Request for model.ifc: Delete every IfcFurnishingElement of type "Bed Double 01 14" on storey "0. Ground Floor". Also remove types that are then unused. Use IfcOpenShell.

First a look at what the model holds.

```python
import ifcopenshell
import ifcopenshell.util.element

model = ifcopenshell.open("model.ifc")
print(model.schema)
storey = next(s for s in model.by_type("IfcBuildingStorey") if s.Name == "0. Ground Floor")
furniture = [e for e in ifcopenshell.util.element.get_decomposition(storey) if e.is_a("IfcFurnishingElement")]
seen = {}
for e in furniture:
    element_type = ifcopenshell.util.element.get_type(e)
    name = element_type.Name if element_type not in (None, e) else None
    seen[name] = seen.get(name, 0) + 1
for name, count in sorted(seen.items(), key=str):
    print(count, "x", name)
```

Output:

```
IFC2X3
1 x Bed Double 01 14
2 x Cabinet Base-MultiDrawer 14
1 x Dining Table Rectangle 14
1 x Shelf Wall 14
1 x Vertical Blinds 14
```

```python
import ifcopenshell
import ifcopenshell.api.root
import ifcopenshell.util.element

model = ifcopenshell.open("model.ifc")

storey = next(s for s in model.by_type("IfcBuildingStorey") if s.Name == "0. Ground Floor")
furniture = [e for e in ifcopenshell.util.element.get_decomposition(storey) if e.is_a("IfcFurnishingElement")]
targets = [e for e in furniture if (t := ifcopenshell.util.element.get_type(e)) not in (None, e) and t.Name == "Bed Double 01 14"]
types = {ifcopenshell.util.element.get_type(e) for e in targets} - {None, *targets}

for e in targets:
    ifcopenshell.api.root.remove_product(model, product=e)
print(len(targets), "removed")

unused = [t for t in types if not ifcopenshell.util.element.get_types(t)]
for t in unused:
    ifcopenshell.api.root.remove_product(model, product=t)
print(len(unused), "unused types removed")

model.write("model-out.ifc")
```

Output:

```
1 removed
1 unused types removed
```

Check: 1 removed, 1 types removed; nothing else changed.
